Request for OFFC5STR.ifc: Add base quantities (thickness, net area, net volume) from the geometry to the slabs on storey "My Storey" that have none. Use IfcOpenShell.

First a look at what the model holds.

```python
import ifcopenshell
import ifcopenshell.util.element
import ifcopenshell.util.unit

model = ifcopenshell.open("OFFC5STR.ifc")
print(model.schema)
for unit_type in ("LENGTHUNIT", "AREAUNIT", "VOLUMEUNIT"):
    print(unit_type, ifcopenshell.util.unit.calculate_unit_scale(model, unit_type))
storey = next(s for s in model.by_type("IfcBuildingStorey") if s.Name == "My Storey")
slabs = [e for e in ifcopenshell.util.element.get_decomposition(storey) if e.is_a("IfcSlab")]
for e in sorted(slabs, key=lambda e: e.id()):
    print(e.id(), e.is_a(), e.Name, list(ifcopenshell.util.element.get_psets(e, qtos_only=True)), sep=" | ")
```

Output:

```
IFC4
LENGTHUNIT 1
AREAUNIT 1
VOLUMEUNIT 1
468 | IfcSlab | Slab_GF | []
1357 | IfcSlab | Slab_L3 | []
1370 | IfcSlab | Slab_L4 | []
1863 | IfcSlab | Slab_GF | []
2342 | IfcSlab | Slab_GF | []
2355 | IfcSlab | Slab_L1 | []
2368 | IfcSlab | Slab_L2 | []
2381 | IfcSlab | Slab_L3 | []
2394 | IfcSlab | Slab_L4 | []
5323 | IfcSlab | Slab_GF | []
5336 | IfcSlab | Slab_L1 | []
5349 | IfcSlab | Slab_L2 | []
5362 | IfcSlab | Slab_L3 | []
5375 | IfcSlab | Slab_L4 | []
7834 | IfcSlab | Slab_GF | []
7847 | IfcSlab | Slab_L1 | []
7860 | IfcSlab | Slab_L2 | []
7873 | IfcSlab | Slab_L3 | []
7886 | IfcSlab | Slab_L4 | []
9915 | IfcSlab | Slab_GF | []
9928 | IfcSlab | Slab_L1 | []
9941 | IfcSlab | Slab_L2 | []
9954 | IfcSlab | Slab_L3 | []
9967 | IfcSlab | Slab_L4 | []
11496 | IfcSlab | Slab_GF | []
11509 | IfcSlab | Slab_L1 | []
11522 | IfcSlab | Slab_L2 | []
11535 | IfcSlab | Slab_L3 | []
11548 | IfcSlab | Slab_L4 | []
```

```python
import ifcopenshell
import ifcopenshell.api.pset
import ifcopenshell.geom
import ifcopenshell.util.element
import ifcopenshell.util.shape
import ifcopenshell.util.unit

model = ifcopenshell.open("OFFC5STR.ifc")
unit_scale = ifcopenshell.util.unit.calculate_unit_scale(model)
area_scale = ifcopenshell.util.unit.calculate_unit_scale(model, "AREAUNIT")
volume_scale = ifcopenshell.util.unit.calculate_unit_scale(model, "VOLUMEUNIT")
settings = ifcopenshell.geom.settings()

storey = next(s for s in model.by_type("IfcBuildingStorey") if s.Name == "My Storey")
slabs = [e for e in ifcopenshell.util.element.get_decomposition(storey) if e.is_a("IfcSlab")]

for e in sorted(slabs, key=lambda e: e.id()):
    if ifcopenshell.util.element.get_psets(e, qtos_only=True, should_inherit=False):
        continue
    # Geometry comes back in metres, in the element's own axes.
    shape = ifcopenshell.geom.create_shape(settings, e)
    values = {
        "Width": ifcopenshell.util.shape.get_z(shape.geometry) / unit_scale,
        "NetArea": ifcopenshell.util.shape.get_footprint_area(shape.geometry) / area_scale,
        "NetVolume": ifcopenshell.util.shape.get_volume(shape.geometry) / volume_scale,
    }
    qto = ifcopenshell.api.pset.add_qto(model, product=e, name="Qto_SlabBaseQuantities")
    ifcopenshell.api.pset.edit_qto(model, qto=qto, properties=values)
    print(e.id(), {k: round(v, 3) for k, v in values.items()})

model.write("OFFC5STR_edited.ifc")
```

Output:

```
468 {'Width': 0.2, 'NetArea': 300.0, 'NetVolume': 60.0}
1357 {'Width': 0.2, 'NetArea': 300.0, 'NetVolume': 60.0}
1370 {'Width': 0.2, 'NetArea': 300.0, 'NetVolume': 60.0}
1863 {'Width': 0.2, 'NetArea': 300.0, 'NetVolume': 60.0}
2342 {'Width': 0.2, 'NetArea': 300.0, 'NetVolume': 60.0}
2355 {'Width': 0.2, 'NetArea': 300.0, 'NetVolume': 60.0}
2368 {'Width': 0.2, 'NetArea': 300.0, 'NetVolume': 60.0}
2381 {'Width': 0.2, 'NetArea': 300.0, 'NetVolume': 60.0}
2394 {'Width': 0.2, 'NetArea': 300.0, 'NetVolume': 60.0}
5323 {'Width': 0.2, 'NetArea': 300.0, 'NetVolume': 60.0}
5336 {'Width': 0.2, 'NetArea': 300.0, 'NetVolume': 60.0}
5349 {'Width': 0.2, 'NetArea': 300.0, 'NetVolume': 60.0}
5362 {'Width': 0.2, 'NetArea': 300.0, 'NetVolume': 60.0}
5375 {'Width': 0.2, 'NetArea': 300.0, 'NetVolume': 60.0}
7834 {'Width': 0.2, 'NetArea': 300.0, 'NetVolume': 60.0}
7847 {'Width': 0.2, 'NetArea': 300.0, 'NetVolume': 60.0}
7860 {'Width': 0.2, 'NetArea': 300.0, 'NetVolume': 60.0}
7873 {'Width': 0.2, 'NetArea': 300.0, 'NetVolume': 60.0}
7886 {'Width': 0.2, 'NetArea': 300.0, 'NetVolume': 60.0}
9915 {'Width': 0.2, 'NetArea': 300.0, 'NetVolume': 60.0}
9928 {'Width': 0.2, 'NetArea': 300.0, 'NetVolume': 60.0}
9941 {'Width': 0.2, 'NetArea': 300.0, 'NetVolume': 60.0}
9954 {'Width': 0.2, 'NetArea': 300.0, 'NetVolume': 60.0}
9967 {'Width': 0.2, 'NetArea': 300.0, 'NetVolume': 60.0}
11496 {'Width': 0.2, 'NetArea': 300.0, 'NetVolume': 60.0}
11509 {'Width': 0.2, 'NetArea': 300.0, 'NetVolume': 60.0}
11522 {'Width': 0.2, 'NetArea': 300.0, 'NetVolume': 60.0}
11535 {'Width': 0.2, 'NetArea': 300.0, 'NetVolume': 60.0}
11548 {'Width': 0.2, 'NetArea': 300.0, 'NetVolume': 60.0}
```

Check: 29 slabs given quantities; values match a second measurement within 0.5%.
